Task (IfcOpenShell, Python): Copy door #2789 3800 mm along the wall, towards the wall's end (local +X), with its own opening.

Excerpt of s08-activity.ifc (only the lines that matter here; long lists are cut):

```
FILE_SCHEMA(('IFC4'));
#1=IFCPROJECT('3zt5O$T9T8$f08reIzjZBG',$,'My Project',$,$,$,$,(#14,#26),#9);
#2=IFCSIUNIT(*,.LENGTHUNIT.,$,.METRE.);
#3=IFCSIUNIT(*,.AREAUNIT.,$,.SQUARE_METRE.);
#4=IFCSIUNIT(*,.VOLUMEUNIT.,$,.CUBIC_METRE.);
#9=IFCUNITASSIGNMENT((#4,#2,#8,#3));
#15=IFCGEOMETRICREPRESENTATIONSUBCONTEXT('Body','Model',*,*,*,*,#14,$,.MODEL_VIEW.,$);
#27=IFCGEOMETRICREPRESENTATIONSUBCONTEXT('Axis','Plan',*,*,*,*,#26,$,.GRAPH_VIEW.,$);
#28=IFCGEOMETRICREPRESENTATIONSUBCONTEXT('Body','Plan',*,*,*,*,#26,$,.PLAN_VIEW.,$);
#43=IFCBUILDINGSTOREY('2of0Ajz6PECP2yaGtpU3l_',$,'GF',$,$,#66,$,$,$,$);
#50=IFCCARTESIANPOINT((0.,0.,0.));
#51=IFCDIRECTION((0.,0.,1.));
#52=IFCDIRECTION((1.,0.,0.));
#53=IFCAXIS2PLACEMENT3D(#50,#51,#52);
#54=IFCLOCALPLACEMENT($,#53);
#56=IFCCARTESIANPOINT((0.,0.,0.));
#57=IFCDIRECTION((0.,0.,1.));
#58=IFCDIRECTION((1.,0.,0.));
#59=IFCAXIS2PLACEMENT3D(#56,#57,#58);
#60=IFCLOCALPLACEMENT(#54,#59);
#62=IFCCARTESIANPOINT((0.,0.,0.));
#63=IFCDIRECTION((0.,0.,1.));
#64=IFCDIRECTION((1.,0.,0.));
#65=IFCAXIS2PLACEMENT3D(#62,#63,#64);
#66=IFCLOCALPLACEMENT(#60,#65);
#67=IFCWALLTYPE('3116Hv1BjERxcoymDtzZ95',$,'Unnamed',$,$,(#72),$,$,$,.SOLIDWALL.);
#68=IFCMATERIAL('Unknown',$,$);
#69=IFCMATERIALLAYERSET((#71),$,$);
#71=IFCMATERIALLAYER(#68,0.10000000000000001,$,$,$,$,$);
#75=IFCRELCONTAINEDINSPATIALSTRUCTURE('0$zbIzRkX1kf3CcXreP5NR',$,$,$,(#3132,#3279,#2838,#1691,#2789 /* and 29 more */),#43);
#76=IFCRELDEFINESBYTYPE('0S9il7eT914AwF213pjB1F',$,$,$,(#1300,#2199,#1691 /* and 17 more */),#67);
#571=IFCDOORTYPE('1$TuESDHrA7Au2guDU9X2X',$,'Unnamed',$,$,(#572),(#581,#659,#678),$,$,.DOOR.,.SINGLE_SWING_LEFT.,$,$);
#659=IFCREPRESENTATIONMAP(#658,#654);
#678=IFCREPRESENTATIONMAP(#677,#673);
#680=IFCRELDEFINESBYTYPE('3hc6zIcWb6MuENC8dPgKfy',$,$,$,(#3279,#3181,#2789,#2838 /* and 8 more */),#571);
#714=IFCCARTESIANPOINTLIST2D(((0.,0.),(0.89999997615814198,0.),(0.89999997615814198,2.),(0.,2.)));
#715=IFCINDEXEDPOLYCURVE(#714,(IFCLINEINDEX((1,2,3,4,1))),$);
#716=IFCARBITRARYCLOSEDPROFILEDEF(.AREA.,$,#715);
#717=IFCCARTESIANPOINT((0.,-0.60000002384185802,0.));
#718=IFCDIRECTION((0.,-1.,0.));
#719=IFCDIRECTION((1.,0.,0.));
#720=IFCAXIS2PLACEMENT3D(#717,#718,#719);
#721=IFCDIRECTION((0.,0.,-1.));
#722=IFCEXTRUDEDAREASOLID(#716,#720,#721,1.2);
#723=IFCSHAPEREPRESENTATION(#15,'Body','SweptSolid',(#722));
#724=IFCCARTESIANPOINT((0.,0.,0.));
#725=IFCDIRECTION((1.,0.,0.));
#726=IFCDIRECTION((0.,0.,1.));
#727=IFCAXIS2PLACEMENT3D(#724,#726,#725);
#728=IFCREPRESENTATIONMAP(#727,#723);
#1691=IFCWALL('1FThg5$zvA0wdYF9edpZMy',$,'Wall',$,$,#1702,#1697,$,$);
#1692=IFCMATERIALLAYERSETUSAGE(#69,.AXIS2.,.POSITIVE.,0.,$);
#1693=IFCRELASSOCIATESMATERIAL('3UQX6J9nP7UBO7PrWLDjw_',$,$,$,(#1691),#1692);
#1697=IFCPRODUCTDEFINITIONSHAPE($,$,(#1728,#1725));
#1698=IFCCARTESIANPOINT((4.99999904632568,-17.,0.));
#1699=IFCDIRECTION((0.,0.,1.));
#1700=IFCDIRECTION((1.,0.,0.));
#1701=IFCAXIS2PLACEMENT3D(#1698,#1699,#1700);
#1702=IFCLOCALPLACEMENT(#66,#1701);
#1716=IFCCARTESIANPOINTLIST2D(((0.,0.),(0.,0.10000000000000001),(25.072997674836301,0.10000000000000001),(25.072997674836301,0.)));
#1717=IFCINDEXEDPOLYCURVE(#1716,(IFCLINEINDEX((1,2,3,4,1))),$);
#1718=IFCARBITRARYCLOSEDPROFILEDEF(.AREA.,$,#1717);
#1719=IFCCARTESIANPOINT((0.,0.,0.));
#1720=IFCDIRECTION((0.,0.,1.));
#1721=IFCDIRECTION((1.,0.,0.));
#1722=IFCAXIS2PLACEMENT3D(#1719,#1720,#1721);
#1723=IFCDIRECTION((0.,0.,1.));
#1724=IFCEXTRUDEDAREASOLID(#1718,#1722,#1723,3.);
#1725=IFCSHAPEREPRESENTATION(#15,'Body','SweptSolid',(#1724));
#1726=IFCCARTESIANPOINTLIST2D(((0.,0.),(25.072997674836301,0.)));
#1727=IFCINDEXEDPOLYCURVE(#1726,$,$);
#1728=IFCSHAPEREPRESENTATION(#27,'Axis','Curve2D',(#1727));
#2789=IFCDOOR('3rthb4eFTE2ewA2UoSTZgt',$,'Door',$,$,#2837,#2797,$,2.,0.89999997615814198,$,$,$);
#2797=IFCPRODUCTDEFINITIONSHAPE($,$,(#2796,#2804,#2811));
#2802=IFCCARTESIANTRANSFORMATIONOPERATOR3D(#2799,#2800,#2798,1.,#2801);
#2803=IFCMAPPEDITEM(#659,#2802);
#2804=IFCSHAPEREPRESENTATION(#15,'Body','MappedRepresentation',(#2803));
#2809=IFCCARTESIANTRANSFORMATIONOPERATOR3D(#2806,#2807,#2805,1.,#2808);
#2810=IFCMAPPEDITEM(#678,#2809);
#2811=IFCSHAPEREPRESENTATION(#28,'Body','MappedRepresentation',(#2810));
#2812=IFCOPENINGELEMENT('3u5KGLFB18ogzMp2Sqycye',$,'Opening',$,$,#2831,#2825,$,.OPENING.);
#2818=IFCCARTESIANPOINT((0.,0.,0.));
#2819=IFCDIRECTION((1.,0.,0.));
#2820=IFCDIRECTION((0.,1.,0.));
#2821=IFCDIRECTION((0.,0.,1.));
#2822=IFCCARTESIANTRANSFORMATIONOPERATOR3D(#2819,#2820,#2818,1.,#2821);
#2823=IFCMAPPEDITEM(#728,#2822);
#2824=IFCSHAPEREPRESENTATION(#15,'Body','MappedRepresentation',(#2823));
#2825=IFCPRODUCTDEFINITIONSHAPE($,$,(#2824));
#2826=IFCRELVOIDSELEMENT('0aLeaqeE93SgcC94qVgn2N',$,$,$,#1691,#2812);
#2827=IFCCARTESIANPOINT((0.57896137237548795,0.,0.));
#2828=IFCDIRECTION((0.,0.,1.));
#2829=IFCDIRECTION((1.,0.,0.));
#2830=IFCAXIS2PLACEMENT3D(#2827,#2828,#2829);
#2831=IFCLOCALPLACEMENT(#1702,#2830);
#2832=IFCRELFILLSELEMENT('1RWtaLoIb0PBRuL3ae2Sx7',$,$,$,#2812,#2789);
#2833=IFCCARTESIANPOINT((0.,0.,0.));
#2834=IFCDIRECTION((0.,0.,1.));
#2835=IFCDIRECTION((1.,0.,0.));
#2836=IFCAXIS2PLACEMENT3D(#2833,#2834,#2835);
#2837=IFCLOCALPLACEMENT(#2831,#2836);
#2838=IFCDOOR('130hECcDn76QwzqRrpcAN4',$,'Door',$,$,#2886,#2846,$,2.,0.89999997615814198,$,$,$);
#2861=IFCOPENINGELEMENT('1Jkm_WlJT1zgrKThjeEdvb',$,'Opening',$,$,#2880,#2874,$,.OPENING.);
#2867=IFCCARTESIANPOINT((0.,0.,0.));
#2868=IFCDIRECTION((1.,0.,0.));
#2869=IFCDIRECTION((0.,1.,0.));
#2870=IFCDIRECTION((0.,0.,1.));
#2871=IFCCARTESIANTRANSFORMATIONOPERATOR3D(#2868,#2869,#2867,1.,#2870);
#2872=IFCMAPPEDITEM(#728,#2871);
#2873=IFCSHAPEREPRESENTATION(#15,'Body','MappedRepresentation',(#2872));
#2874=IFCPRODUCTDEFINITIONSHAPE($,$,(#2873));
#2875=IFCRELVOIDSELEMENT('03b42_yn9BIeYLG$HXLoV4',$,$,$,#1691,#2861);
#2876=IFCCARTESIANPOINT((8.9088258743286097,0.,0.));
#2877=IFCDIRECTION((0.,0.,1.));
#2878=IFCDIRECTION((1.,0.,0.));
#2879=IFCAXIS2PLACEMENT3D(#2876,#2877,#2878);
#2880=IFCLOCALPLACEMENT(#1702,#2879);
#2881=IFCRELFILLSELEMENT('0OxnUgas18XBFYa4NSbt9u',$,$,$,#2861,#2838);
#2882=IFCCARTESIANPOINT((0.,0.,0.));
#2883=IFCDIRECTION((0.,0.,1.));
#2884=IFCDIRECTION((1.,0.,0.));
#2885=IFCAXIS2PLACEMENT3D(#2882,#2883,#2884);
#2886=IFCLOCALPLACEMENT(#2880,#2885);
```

```python
import ifcopenshell
import ifcopenshell.api.feature
import ifcopenshell.api.geometry
import ifcopenshell.api.root
import ifcopenshell.geom
import ifcopenshell.util.element
import ifcopenshell.util.placement
import ifcopenshell.util.shape
import ifcopenshell.util.unit

model = ifcopenshell.open("s08-activity.ifc")
unit_scale = ifcopenshell.util.unit.calculate_unit_scale(model)
settings = ifcopenshell.geom.settings()


def volume(element):
    """Net volume in cubic metres, openings subtracted."""
    shape = ifcopenshell.geom.create_shape(settings, element)
    return ifcopenshell.util.shape.get_volume(shape.geometry)


door = model.by_guid("3rthb4eFTE2ewA2UoSTZgt")
opening = door.FillsVoids[0].RelatingOpeningElement
wall = opening.VoidsElements[0].RelatingBuildingElement
before = volume(wall)
shift = ifcopenshell.util.placement.get_local_placement(wall.ObjectPlacement)[:3, 0] * 3.8 / unit_scale

# copy_class copies the void relationship, type, container and properties, but no geometry.
new_opening = ifcopenshell.api.root.copy_class(model, product=opening)
new_opening.Representation = ifcopenshell.util.element.copy_deep(
    model, opening.Representation, exclude=["IfcGeometricRepresentationContext", "IfcRepresentationMap"]
)
new_door = ifcopenshell.api.root.copy_class(model, product=door)
new_door.Representation = ifcopenshell.util.element.copy_deep(
    model, door.Representation, exclude=["IfcGeometricRepresentationContext", "IfcRepresentationMap"]
)
ifcopenshell.api.feature.add_filling(model, opening=new_opening, element=new_door)

for old, new in ((opening, new_opening), (door, new_door)):
    matrix = ifcopenshell.util.placement.get_local_placement(old.ObjectPlacement)
    matrix[:3, 3] += shift
    ifcopenshell.api.geometry.edit_object_placement(model, product=new, matrix=matrix, is_si=False)

after = volume(wall)

print(f"wall volume {before:.3f} -> {after:.3f} m3")

model.write("s08-activity_rev.ifc")
```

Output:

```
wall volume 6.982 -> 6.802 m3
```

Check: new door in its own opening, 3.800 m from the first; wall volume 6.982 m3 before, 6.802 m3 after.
